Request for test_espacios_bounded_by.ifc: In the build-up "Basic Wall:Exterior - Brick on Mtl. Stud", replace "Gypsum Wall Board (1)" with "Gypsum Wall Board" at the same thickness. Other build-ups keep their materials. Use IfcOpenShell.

First a look at what the model holds.

```python
import ifcopenshell
import ifcopenshell.util.element

model = ifcopenshell.open("test_espacios_bounded_by.ifc")
print(model.schema)
for layer_set in model.by_type("IfcMaterialLayerSet"):
    if layer_set.LayerSetName == "Basic Wall:Exterior - Brick on Mtl. Stud":
        for layer in layer_set.MaterialLayers:
            print(layer.id(), layer.Material and layer.Material.Name, layer.LayerThickness, sep=" | ")
        print(len(ifcopenshell.util.element.get_elements_by_material(model, layer_set)), "elements and types use it")
print(sorted(m.Name for m in model.by_type("IfcMaterial") if m.Name)[:60])
```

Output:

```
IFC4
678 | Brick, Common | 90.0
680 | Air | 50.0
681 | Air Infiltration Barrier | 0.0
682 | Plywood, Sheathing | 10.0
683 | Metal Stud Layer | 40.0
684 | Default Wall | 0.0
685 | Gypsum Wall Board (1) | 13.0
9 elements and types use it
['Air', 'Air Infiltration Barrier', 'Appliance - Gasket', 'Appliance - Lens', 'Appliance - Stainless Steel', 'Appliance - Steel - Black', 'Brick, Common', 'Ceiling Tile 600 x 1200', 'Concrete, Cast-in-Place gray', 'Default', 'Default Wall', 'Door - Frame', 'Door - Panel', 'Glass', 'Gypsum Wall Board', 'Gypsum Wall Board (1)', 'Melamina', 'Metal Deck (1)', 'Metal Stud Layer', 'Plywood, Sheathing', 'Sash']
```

```python
import ifcopenshell
import ifcopenshell.api.material

model = ifcopenshell.open("test_espacios_bounded_by.ifc")

layer_set = next(s for s in model.by_type("IfcMaterialLayerSet") if s.LayerSetName == "Basic Wall:Exterior - Brick on Mtl. Stud")
layer = next(l for l in layer_set.MaterialLayers if l.Material and l.Material.Name == "Gypsum Wall Board (1)")
material = next(m for m in model.by_type("IfcMaterial") if m.Name == "Gypsum Wall Board")

# Point this one layer at the other material; renaming the old one would change it everywhere.
ifcopenshell.api.material.edit_layer(model, layer=layer, attributes={"Name": material.Name}, material=material)

print([l.Material.Name if l.Material else None for l in layer_set.MaterialLayers])

model.write("test_espacios_bounded_by-out.ifc")
```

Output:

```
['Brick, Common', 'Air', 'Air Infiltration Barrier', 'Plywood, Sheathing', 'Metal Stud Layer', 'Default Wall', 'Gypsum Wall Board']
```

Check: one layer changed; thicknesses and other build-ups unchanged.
